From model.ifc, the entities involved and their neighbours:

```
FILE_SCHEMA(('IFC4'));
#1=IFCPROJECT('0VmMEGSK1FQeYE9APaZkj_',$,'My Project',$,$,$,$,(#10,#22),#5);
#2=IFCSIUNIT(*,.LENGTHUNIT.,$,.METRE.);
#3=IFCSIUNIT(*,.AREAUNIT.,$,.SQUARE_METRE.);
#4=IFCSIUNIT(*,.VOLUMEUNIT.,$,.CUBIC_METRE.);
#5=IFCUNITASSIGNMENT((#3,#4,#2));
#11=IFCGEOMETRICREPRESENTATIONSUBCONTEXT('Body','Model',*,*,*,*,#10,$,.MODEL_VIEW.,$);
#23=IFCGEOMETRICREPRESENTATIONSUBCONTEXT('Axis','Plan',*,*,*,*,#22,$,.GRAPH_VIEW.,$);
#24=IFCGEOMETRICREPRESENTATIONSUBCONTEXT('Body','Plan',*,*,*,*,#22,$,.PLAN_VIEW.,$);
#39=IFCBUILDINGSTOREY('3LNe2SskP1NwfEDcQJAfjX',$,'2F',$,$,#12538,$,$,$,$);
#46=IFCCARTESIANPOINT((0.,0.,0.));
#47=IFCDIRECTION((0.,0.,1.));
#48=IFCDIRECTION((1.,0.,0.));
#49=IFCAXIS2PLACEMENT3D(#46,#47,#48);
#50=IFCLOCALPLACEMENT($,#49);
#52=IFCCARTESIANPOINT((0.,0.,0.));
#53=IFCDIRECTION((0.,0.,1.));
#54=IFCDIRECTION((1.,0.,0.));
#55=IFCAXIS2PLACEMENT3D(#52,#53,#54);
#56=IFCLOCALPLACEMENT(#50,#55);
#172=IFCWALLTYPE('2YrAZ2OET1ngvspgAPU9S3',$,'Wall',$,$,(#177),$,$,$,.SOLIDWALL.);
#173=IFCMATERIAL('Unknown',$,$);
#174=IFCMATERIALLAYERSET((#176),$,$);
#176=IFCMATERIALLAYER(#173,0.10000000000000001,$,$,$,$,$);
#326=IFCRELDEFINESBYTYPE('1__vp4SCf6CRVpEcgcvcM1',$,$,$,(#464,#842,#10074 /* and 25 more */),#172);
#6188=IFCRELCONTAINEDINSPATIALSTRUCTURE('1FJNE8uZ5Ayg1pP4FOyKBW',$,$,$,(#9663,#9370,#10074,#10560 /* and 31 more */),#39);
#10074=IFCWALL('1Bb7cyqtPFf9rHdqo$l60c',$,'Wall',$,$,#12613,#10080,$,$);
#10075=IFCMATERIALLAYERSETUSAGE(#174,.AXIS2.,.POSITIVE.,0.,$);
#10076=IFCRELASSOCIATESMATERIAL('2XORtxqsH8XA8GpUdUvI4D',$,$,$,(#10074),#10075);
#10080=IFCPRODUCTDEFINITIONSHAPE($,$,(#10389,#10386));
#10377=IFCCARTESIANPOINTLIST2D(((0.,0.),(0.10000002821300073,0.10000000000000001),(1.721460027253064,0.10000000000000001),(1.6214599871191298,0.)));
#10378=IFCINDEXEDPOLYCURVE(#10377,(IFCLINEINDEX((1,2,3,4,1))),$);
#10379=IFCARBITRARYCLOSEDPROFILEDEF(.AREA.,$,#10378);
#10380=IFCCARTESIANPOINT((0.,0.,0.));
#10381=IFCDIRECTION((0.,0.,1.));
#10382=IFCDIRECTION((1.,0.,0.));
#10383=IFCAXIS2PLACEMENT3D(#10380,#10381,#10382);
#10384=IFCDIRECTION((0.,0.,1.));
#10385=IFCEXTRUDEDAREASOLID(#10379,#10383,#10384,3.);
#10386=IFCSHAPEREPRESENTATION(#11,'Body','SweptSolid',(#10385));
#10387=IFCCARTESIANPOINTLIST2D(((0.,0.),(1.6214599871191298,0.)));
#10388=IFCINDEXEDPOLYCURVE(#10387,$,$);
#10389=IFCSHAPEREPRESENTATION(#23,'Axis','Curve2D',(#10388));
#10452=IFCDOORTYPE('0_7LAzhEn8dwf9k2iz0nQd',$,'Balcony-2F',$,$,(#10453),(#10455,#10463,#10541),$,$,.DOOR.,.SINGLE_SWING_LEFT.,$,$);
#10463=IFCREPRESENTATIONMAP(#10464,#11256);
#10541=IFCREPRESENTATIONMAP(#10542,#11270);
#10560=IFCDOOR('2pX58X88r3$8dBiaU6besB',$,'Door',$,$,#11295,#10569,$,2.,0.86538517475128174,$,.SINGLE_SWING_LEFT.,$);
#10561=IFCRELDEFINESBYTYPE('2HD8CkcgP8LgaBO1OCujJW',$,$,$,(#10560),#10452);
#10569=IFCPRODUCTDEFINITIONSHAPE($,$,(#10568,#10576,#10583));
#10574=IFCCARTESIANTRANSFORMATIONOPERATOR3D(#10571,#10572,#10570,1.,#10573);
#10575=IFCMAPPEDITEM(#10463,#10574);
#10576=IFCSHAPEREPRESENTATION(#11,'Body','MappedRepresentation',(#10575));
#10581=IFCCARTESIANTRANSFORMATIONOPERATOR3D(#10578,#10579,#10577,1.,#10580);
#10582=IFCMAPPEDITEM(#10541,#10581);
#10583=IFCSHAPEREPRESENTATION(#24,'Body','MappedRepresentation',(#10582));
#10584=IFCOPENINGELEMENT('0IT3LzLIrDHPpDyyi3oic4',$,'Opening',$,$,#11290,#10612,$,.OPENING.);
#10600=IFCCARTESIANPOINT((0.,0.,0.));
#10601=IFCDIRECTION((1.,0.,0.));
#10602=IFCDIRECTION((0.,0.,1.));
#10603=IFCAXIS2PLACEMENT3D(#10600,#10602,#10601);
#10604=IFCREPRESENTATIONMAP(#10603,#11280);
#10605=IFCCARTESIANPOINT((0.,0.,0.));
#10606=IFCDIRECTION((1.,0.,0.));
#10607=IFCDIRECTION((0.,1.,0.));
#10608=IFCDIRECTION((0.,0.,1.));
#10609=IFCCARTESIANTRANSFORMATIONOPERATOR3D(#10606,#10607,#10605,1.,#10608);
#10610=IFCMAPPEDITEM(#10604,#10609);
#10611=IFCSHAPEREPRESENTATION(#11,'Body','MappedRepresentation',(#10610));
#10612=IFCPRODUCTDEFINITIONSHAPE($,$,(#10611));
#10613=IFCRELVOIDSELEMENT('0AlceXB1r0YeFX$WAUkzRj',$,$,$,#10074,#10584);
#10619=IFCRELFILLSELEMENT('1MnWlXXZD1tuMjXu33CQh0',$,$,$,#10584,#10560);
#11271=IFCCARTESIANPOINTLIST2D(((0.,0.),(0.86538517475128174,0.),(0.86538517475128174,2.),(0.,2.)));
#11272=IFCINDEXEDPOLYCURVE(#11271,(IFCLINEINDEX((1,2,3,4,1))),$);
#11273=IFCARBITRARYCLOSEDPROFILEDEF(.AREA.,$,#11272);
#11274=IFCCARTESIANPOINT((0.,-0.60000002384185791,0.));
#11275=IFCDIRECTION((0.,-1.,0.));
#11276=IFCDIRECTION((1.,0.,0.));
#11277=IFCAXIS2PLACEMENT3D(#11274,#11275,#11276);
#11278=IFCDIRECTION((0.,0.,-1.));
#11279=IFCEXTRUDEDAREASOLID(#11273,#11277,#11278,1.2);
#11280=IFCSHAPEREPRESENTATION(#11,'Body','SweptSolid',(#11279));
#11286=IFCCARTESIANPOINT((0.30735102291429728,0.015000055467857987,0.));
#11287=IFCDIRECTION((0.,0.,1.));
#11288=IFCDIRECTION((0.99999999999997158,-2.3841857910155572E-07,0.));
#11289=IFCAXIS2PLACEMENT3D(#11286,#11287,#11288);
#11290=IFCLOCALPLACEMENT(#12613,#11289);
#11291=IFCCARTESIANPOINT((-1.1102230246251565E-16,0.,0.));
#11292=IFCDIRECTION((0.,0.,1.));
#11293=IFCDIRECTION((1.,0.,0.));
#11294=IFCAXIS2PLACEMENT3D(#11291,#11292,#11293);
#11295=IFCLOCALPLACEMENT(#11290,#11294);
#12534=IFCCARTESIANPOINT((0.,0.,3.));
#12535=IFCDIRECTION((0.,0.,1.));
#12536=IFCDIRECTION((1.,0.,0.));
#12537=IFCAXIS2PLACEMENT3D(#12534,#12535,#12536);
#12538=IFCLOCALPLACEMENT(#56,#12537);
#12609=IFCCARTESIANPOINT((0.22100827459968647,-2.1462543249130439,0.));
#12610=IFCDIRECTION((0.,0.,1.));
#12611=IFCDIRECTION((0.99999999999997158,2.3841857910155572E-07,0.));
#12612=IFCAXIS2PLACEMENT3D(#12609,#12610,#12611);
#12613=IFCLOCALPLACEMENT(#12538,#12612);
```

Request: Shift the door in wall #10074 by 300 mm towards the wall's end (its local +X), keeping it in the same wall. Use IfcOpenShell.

```python
import ifcopenshell
import ifcopenshell.api.geometry
import ifcopenshell.util.placement
import ifcopenshell.util.unit

model = ifcopenshell.open("model.ifc")
unit_scale = ifcopenshell.util.unit.calculate_unit_scale(model)

door = model.by_id(10560)
opening = door.FillsVoids[0].RelatingOpeningElement
wall = opening.VoidsElements[0].RelatingBuildingElement

wall_matrix = ifcopenshell.util.placement.get_local_placement(wall.ObjectPlacement)
shift = wall_matrix[:3, 0] * 0.3 / unit_scale
before = ifcopenshell.util.placement.get_local_placement(door.ObjectPlacement)[:3, 3].copy()

# The door is placed relative to its opening, so it follows when the opening moves.
matrix = ifcopenshell.util.placement.get_local_placement(opening.ObjectPlacement)
matrix[:3, 3] += shift
ifcopenshell.api.geometry.edit_object_placement(
    model, product=opening, matrix=matrix, is_si=False, should_transform_children=True
)

after = ifcopenshell.util.placement.get_local_placement(door.ObjectPlacement)[:3, 3]
print("door moved by", (after - before).round(3) + 0.0)

model.write("model_v2.ifc")
```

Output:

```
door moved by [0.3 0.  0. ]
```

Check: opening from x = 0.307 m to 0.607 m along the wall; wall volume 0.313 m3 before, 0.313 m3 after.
